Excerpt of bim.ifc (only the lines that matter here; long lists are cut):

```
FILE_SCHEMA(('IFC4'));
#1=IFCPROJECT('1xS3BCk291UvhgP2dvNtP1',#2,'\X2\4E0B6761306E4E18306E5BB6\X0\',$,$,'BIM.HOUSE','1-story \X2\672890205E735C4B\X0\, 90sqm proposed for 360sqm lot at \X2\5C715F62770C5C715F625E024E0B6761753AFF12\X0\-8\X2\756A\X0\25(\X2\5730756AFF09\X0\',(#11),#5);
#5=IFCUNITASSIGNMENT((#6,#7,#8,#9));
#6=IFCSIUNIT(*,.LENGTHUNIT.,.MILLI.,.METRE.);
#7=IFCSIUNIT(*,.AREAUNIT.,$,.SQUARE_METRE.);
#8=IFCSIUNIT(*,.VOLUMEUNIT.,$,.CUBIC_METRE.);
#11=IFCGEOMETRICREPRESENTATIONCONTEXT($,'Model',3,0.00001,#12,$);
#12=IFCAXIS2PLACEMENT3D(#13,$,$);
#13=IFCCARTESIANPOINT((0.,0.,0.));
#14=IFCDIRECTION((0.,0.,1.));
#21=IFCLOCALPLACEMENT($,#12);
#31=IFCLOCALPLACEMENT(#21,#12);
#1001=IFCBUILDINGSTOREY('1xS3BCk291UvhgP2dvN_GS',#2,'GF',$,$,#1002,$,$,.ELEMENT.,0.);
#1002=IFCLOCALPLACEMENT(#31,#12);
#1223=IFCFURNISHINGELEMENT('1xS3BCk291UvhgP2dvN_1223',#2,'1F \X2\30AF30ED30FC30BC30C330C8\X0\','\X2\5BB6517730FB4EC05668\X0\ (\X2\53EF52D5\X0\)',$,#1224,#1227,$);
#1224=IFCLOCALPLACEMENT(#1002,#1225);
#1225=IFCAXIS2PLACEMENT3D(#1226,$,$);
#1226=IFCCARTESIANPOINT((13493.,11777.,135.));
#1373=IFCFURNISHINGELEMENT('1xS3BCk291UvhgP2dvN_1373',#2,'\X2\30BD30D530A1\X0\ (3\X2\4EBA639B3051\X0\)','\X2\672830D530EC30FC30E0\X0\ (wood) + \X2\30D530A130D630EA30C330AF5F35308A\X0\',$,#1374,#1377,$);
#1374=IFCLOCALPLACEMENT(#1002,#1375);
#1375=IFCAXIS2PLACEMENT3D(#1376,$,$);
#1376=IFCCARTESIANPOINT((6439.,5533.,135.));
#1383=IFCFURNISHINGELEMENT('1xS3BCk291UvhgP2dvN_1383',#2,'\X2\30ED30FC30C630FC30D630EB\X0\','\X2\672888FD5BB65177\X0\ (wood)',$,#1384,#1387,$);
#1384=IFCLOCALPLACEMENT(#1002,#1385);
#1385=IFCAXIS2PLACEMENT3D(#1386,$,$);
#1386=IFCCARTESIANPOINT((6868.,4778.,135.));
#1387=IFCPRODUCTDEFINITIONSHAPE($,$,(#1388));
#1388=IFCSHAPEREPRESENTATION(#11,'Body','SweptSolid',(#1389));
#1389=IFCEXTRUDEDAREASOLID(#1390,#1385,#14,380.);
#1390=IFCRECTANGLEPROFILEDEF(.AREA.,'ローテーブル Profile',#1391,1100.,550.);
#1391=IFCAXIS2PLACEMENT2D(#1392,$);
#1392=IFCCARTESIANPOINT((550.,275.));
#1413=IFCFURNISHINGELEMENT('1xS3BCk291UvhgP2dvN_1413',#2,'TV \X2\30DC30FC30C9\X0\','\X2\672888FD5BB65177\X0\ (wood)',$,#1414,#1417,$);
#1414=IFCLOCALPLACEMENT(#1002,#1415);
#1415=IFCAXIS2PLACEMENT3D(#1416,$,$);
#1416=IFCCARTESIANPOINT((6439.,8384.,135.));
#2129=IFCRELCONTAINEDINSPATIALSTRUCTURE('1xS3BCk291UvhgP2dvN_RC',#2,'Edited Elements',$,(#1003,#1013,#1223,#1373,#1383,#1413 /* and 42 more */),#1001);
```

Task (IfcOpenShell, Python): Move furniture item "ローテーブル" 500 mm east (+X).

```python
import ifcopenshell
import ifcopenshell.api.geometry
import ifcopenshell.util.placement
import ifcopenshell.util.unit

model = ifcopenshell.open("bim.ifc")
unit_scale = ifcopenshell.util.unit.calculate_unit_scale(model)

item = model.by_id(1383)
matrix = ifcopenshell.util.placement.get_local_placement(item.ObjectPlacement)
matrix[0, 3] += 0.5 / unit_scale
ifcopenshell.api.geometry.edit_object_placement(model, product=item, matrix=matrix, is_si=False)

print(ifcopenshell.util.placement.get_local_placement(item.ObjectPlacement).round(3) + 0.0)

model.write("bim_edited.ifc")
```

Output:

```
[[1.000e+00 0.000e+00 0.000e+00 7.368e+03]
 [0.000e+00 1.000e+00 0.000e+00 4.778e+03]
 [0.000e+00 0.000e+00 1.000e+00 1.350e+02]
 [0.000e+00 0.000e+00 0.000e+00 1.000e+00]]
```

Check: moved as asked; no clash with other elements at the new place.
